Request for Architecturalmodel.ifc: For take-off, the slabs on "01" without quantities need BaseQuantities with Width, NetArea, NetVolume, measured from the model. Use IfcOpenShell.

First a look at what the model holds.

```python
import ifcopenshell
import ifcopenshell.util.element
import ifcopenshell.util.unit

model = ifcopenshell.open("Architecturalmodel.ifc")
print(model.schema)
for unit_type in ("LENGTHUNIT", "AREAUNIT", "VOLUMEUNIT"):
    print(unit_type, ifcopenshell.util.unit.calculate_unit_scale(model, unit_type))
storey = next(s for s in model.by_type("IfcBuildingStorey") if s.Name == "01")
slabs = [e for e in ifcopenshell.util.element.get_decomposition(storey) if e.is_a("IfcSlab")]
for e in sorted(slabs, key=lambda e: e.id()):
    print(e.id(), e.is_a(), e.Name, list(ifcopenshell.util.element.get_psets(e, qtos_only=True)), sep=" | ")
```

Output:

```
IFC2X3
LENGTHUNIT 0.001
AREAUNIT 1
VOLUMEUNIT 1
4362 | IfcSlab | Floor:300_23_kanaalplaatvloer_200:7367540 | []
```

```python
import ifcopenshell
import ifcopenshell.api.pset
import ifcopenshell.geom
import ifcopenshell.util.element
import ifcopenshell.util.shape
import ifcopenshell.util.unit

model = ifcopenshell.open("Architecturalmodel.ifc")
unit_scale = ifcopenshell.util.unit.calculate_unit_scale(model)
area_scale = ifcopenshell.util.unit.calculate_unit_scale(model, "AREAUNIT")
volume_scale = ifcopenshell.util.unit.calculate_unit_scale(model, "VOLUMEUNIT")
settings = ifcopenshell.geom.settings()

storey = next(s for s in model.by_type("IfcBuildingStorey") if s.Name == "01")
slabs = [e for e in ifcopenshell.util.element.get_decomposition(storey) if e.is_a("IfcSlab")]

for e in sorted(slabs, key=lambda e: e.id()):
    if ifcopenshell.util.element.get_psets(e, qtos_only=True, should_inherit=False):
        continue
    # Geometry comes back in metres, in the element's own axes.
    shape = ifcopenshell.geom.create_shape(settings, e)
    values = {
        "Width": ifcopenshell.util.shape.get_z(shape.geometry) / unit_scale,
        "NetArea": ifcopenshell.util.shape.get_footprint_area(shape.geometry) / area_scale,
        "NetVolume": ifcopenshell.util.shape.get_volume(shape.geometry) / volume_scale,
    }
    qto = ifcopenshell.api.pset.add_qto(model, product=e, name="BaseQuantities")
    ifcopenshell.api.pset.edit_qto(model, qto=qto, properties=values)
    print(e.id(), {k: round(v, 3) for k, v in values.items()})

model.write("Architecturalmodel_edited.ifc")
```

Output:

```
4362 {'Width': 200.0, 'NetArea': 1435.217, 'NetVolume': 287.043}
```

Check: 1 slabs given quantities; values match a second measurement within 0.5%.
